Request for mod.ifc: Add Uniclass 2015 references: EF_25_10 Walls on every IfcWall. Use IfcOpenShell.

First a look at what the model holds.

```python
import ifcopenshell

model = ifcopenshell.open("mod.ifc")
print(model.schema)
print("classifications:", [c.Name for c in model.by_type("IfcClassification")])
for ifc_class in ("IfcDoor", "IfcRoof", "IfcStair", "IfcWall", "IfcWindow"):
    print(ifc_class, len(model.by_type(ifc_class)))
```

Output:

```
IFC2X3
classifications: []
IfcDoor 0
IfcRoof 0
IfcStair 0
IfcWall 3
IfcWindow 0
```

```python
import ifcopenshell
import ifcopenshell.api.classification

model = ifcopenshell.open("mod.ifc")

# IFC2X3 requires Source and Edition and has no link from the project to the system.
system = model.create_entity("IfcClassification", Source="NBS", Edition="2015", Name="Uniclass 2015")

codes = {
    "IfcWall": ("EF_25_10", "Walls"),
}
for ifc_class, (code, name) in codes.items():
    products = model.by_type(ifc_class)
    ifcopenshell.api.classification.add_reference(
        model, products=products, classification=system, identification=code, name=name
    )
    print(code, len(products))

model.write("mod_updated.ifc")
```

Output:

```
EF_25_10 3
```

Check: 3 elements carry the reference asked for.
